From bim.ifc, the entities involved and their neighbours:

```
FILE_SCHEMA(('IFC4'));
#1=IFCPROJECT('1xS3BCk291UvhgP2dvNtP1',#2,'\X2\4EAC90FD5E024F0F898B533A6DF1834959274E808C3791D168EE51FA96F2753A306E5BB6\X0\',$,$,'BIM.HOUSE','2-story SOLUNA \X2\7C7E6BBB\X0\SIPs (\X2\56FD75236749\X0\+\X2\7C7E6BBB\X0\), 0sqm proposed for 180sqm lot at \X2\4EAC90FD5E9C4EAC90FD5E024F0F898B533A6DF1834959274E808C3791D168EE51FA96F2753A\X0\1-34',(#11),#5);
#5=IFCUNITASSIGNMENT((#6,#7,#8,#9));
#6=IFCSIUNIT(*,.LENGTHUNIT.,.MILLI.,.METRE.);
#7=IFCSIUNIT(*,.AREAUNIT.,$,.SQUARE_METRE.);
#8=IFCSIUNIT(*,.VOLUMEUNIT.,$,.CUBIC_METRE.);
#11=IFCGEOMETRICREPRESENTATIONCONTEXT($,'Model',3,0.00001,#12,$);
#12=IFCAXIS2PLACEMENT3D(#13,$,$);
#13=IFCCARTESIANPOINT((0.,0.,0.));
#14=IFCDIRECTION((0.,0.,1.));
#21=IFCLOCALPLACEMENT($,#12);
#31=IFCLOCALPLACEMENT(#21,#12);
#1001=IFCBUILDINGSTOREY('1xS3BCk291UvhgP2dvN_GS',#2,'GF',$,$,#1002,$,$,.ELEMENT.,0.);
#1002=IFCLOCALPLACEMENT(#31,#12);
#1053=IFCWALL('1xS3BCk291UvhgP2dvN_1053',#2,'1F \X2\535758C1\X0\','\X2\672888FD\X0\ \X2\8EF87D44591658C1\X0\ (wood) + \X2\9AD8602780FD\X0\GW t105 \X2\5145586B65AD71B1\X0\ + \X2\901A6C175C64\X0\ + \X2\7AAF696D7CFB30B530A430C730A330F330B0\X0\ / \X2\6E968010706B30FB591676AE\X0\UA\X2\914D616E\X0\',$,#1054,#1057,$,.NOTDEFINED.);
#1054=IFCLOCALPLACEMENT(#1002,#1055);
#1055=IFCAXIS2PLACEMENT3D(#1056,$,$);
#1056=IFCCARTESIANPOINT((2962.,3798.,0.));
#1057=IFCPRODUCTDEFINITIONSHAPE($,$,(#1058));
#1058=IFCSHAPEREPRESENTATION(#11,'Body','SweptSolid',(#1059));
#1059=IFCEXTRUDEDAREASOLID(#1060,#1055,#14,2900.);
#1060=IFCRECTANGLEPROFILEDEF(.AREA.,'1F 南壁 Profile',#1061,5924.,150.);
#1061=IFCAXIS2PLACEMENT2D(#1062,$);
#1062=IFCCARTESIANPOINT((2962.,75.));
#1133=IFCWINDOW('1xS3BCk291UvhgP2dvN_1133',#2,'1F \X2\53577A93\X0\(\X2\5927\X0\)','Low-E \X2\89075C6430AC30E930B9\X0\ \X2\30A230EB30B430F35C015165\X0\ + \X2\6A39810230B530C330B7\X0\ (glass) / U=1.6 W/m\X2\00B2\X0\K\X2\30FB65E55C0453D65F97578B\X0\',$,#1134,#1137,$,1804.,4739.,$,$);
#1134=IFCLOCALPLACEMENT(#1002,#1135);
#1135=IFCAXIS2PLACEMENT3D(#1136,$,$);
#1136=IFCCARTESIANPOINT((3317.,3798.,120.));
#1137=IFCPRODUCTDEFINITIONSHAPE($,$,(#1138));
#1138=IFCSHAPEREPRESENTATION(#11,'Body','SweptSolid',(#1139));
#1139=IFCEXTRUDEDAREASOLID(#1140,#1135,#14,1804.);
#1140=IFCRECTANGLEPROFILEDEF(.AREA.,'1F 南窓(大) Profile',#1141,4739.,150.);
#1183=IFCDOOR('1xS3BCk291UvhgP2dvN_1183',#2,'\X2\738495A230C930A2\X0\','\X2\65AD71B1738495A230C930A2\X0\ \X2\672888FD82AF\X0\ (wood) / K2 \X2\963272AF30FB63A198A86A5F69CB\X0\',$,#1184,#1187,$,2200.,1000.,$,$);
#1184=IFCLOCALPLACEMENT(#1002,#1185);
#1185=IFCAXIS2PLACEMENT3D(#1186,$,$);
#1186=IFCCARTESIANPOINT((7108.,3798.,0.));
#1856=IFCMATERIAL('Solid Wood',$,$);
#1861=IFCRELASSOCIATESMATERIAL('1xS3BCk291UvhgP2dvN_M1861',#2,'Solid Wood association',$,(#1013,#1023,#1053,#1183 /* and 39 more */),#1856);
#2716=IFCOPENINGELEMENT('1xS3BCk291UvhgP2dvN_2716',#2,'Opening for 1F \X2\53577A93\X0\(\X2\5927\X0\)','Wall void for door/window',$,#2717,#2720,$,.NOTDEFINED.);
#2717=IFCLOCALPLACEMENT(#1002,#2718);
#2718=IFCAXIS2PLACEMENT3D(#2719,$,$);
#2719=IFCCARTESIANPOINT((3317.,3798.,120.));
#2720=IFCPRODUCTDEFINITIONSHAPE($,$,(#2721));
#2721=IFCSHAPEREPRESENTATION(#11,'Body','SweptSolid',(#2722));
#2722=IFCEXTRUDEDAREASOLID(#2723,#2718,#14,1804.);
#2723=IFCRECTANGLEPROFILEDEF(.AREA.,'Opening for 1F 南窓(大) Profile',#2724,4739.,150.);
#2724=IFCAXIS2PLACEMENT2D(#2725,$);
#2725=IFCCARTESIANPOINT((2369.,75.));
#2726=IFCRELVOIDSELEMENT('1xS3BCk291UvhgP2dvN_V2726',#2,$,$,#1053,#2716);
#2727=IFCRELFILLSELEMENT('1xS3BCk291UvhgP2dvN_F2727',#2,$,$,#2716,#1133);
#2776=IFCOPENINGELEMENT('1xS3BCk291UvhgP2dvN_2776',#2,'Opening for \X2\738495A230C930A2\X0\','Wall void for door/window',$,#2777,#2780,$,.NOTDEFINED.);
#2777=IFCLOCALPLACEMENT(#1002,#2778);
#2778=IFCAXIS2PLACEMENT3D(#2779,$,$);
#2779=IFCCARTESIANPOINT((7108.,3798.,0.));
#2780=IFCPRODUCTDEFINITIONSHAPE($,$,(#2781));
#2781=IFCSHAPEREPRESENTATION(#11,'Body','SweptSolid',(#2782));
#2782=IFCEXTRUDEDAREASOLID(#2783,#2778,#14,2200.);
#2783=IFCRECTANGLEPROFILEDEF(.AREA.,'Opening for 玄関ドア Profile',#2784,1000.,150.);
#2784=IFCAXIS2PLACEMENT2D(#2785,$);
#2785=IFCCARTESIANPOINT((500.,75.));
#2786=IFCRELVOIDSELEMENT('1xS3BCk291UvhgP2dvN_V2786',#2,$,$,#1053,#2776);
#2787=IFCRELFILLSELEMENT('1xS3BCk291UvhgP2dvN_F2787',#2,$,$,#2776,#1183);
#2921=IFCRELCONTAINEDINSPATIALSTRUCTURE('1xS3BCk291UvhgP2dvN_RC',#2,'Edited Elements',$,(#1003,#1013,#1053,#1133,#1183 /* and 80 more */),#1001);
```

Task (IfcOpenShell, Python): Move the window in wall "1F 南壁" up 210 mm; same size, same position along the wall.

```python
import numpy as np
import ifcopenshell
import ifcopenshell.api.geometry
import ifcopenshell.util.placement
import ifcopenshell.util.unit

model = ifcopenshell.open("bim.ifc")
unit_scale = ifcopenshell.util.unit.calculate_unit_scale(model)

window = model.by_guid("1xS3BCk291UvhgP2dvN_1133")
opening = window.FillsVoids[0].RelatingOpeningElement
dz = 0.21 / unit_scale

shift = np.array([0.0, 0.0, dz])
# The window is not placed relative to its opening, so move both.
for product in (opening, window):
    matrix = ifcopenshell.util.placement.get_local_placement(product.ObjectPlacement)
    matrix[:3, 3] += shift
    ifcopenshell.api.geometry.edit_object_placement(model, product=product, matrix=matrix, is_si=False)

print(f"moved by {dz * unit_scale:+.3f} m")

model.write("bim_v2.ifc")
```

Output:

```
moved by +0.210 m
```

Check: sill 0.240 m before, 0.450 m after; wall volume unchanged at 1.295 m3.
